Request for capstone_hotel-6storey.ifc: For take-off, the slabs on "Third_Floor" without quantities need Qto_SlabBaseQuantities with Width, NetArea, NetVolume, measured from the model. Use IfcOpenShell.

First a look at what the model holds.

```python
import ifcopenshell
import ifcopenshell.util.element
import ifcopenshell.util.unit

model = ifcopenshell.open("capstone_hotel-6storey.ifc")
print(model.schema)
for unit_type in ("LENGTHUNIT", "AREAUNIT", "VOLUMEUNIT"):
    print(unit_type, ifcopenshell.util.unit.calculate_unit_scale(model, unit_type))
storey = next(s for s in model.by_type("IfcBuildingStorey") if s.Name == "Third_Floor")
slabs = [e for e in ifcopenshell.util.element.get_decomposition(storey) if e.is_a("IfcSlab")]
for e in sorted(slabs, key=lambda e: e.id()):
    print(e.id(), e.is_a(), e.Name, list(ifcopenshell.util.element.get_psets(e, qtos_only=True)), sep=" | ")
```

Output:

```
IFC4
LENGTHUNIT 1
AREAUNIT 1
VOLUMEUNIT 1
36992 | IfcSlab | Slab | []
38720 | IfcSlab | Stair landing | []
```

```python
import ifcopenshell
import ifcopenshell.api.pset
import ifcopenshell.geom
import ifcopenshell.util.element
import ifcopenshell.util.shape
import ifcopenshell.util.unit

model = ifcopenshell.open("capstone_hotel-6storey.ifc")
unit_scale = ifcopenshell.util.unit.calculate_unit_scale(model)
area_scale = ifcopenshell.util.unit.calculate_unit_scale(model, "AREAUNIT")
volume_scale = ifcopenshell.util.unit.calculate_unit_scale(model, "VOLUMEUNIT")
settings = ifcopenshell.geom.settings()

storey = next(s for s in model.by_type("IfcBuildingStorey") if s.Name == "Third_Floor")
slabs = [e for e in ifcopenshell.util.element.get_decomposition(storey) if e.is_a("IfcSlab")]

for e in sorted(slabs, key=lambda e: e.id()):
    if ifcopenshell.util.element.get_psets(e, qtos_only=True, should_inherit=False):
        continue
    # Geometry comes back in metres, in the element's own axes.
    shape = ifcopenshell.geom.create_shape(settings, e)
    values = {
        "Width": ifcopenshell.util.shape.get_z(shape.geometry) / unit_scale,
        "NetArea": ifcopenshell.util.shape.get_footprint_area(shape.geometry) / area_scale,
        "NetVolume": ifcopenshell.util.shape.get_volume(shape.geometry) / volume_scale,
    }
    qto = ifcopenshell.api.pset.add_qto(model, product=e, name="Qto_SlabBaseQuantities")
    ifcopenshell.api.pset.edit_qto(model, qto=qto, properties=values)
    print(e.id(), {k: round(v, 3) for k, v in values.items()})

model.write("capstone_hotel-6storey_rev.ifc")
```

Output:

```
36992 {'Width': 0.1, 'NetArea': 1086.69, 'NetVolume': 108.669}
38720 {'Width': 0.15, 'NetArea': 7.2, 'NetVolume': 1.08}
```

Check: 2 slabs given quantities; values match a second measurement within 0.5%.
